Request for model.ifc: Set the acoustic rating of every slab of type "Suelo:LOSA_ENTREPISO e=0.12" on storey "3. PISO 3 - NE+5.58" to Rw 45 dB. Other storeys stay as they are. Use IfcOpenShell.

First a look at what the model holds.

```python
import ifcopenshell
import ifcopenshell.util.element

model = ifcopenshell.open("model.ifc")
print(model.schema)
storey = next(s for s in model.by_type("IfcBuildingStorey") if s.Name == "3. PISO 3 - NE+5.58")
slabs = [e for e in ifcopenshell.util.element.get_decomposition(storey) if e.is_a("IfcSlab")]
seen = {}
for e in slabs:
    element_type = ifcopenshell.util.element.get_type(e)
    key = (element_type.Name if element_type != e and element_type else None, ifcopenshell.util.element.get_pset(e, "Pset_SlabCommon", "AcousticRating"))
    seen[key] = seen.get(key, 0) + 1
for (name, value), count in sorted(seen.items(), key=str):
    print(count, "x", name, "|", value)
```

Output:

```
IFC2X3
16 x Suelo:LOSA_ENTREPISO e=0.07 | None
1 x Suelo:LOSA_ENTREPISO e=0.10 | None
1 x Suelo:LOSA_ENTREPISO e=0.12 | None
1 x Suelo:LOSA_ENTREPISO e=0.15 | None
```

```python
import ifcopenshell
import ifcopenshell.api.pset
import ifcopenshell.util.element

model = ifcopenshell.open("model.ifc")

storey = next(s for s in model.by_type("IfcBuildingStorey") if s.Name == "3. PISO 3 - NE+5.58")
slabs = [e for e in ifcopenshell.util.element.get_decomposition(storey) if e.is_a("IfcSlab")]

count = 0
for e in slabs:
    element_type = ifcopenshell.util.element.get_type(e)
    if element_type in (None, e) or element_type.Name != "Suelo:LOSA_ENTREPISO e=0.12":
        continue
    # add_pset returns the element's existing set when there is one.
    pset = ifcopenshell.api.pset.add_pset(model, product=e, name="Pset_SlabCommon")
    ifcopenshell.api.pset.edit_pset(model, pset=pset, properties={"AcousticRating": "Rw 45 dB"})
    count += 1

print(count, "slabs updated")

model.write("model_edited.ifc")
```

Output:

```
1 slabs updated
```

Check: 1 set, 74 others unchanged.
